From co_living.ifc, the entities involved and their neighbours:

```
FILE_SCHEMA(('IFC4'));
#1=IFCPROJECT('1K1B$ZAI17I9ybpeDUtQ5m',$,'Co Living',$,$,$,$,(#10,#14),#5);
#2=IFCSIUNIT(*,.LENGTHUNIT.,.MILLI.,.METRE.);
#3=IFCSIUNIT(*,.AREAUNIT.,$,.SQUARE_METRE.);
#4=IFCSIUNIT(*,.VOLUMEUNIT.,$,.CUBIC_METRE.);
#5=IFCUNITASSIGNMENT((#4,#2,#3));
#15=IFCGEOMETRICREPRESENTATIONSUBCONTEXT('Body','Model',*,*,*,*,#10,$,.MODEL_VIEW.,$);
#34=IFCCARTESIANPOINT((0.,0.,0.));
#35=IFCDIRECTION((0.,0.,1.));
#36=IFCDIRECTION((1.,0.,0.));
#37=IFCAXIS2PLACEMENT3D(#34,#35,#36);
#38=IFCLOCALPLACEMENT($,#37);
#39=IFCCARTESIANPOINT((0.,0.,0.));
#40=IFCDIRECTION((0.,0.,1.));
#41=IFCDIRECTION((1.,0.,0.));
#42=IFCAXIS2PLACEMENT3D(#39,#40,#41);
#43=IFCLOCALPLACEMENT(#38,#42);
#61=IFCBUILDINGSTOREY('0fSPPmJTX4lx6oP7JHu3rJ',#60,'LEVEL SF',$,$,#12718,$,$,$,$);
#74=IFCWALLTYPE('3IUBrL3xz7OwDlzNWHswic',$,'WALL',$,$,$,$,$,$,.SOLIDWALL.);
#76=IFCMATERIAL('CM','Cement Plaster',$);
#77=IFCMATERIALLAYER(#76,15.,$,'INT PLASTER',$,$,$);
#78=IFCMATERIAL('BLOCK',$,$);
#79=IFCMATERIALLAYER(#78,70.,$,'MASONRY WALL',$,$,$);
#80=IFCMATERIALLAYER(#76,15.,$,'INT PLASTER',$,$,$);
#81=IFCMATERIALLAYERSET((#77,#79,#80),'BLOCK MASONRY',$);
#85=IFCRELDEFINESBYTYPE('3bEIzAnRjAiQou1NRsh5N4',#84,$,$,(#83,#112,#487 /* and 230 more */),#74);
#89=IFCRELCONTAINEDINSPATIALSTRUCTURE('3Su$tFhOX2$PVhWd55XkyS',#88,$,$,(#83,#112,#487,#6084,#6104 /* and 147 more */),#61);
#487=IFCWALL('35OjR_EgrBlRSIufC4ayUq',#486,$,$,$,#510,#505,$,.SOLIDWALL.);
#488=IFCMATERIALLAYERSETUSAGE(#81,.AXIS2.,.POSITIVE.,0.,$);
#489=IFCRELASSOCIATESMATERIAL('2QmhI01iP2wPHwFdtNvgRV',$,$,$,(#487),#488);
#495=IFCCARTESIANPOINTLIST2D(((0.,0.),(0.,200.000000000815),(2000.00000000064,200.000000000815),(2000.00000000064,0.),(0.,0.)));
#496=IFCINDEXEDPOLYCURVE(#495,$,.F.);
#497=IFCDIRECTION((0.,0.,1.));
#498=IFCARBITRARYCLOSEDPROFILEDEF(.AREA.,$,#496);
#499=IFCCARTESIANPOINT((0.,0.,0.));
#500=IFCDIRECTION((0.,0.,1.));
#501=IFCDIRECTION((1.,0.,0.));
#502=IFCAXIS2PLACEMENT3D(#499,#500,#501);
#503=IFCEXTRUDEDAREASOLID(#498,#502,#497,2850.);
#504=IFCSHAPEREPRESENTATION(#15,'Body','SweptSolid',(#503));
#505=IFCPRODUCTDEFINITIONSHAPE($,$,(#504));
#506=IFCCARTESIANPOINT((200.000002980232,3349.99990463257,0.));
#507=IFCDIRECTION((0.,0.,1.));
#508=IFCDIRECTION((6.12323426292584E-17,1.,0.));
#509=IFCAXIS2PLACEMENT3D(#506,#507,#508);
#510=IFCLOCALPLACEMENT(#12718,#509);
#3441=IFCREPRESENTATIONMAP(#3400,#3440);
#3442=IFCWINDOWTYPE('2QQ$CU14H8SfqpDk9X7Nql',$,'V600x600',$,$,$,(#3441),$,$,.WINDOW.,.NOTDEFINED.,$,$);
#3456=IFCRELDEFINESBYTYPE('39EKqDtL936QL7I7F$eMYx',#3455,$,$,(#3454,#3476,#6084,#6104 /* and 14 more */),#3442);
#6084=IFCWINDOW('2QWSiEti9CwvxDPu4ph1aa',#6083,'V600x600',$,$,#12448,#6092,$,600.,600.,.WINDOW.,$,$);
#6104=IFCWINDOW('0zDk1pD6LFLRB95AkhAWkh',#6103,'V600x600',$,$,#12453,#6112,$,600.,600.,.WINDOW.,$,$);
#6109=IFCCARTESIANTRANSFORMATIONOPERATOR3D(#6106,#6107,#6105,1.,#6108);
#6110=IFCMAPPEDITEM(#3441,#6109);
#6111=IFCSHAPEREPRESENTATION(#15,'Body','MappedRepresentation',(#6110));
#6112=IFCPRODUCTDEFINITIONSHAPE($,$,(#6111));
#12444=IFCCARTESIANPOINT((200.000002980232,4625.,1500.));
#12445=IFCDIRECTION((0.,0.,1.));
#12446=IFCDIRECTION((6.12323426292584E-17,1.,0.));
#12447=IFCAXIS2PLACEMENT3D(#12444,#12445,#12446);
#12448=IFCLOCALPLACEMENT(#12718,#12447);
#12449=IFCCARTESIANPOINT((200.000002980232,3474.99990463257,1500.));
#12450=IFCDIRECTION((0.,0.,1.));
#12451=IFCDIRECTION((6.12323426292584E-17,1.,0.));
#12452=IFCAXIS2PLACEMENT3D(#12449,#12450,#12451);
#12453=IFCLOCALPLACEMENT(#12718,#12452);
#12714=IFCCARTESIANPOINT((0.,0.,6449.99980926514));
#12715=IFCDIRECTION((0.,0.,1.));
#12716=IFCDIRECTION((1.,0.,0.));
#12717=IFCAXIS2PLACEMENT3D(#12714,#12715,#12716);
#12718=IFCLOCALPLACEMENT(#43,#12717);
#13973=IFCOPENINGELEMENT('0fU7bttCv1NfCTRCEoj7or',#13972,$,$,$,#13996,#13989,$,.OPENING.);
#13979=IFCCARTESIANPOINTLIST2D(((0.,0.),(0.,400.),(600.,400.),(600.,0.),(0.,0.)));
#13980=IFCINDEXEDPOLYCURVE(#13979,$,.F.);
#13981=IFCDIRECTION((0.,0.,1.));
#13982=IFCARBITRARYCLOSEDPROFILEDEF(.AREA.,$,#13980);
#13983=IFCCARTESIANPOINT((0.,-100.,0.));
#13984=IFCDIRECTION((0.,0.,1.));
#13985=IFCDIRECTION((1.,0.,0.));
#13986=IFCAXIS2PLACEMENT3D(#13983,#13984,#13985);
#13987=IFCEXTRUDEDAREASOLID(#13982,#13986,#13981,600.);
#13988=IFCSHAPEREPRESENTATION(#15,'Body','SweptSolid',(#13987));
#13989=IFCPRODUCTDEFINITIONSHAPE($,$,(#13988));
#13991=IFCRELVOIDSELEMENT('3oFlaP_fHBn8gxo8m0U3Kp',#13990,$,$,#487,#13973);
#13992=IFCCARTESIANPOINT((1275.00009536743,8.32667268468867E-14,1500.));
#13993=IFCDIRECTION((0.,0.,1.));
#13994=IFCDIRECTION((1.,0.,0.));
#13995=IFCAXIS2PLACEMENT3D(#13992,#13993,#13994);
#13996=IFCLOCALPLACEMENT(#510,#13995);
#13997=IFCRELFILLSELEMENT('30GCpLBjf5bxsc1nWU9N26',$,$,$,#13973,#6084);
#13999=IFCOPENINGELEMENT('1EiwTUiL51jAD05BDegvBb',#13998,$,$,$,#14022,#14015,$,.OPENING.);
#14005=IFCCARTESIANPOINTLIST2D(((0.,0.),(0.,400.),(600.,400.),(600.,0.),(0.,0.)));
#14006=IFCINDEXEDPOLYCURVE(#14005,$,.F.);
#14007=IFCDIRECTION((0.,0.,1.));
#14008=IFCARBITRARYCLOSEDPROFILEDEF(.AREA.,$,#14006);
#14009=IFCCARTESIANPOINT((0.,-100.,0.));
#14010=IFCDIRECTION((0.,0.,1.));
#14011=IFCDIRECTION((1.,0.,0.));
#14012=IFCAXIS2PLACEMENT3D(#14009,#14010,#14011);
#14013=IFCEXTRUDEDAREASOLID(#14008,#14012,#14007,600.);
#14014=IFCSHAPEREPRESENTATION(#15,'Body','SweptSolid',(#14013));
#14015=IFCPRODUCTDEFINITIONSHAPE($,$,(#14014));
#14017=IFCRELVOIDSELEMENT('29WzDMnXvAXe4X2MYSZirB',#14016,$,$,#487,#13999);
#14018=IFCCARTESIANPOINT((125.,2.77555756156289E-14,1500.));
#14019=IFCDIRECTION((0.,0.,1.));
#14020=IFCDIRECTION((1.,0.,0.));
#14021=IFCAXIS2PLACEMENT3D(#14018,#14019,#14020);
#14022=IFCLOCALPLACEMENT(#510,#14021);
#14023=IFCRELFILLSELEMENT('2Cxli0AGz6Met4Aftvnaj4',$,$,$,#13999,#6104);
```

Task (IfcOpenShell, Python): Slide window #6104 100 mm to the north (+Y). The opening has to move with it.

```python
import ifcopenshell
import ifcopenshell.api.geometry
import ifcopenshell.util.placement
import ifcopenshell.util.unit

model = ifcopenshell.open("co_living.ifc")
unit_scale = ifcopenshell.util.unit.calculate_unit_scale(model)

window = model.by_guid("0zDk1pD6LFLRB95AkhAWkh")
opening = window.FillsVoids[0].RelatingOpeningElement
wall = opening.VoidsElements[0].RelatingBuildingElement

wall_matrix = ifcopenshell.util.placement.get_local_placement(wall.ObjectPlacement)
shift = wall_matrix[:3, 0] * 0.1 / unit_scale
before = ifcopenshell.util.placement.get_local_placement(window.ObjectPlacement)[:3, 3].copy()

# The window is not placed relative to its opening, so move both.
for product in (opening, window):
    matrix = ifcopenshell.util.placement.get_local_placement(product.ObjectPlacement)
    matrix[:3, 3] += shift
    ifcopenshell.api.geometry.edit_object_placement(model, product=product, matrix=matrix, is_si=False)

after = ifcopenshell.util.placement.get_local_placement(window.ObjectPlacement)[:3, 3]
print("window moved by", (after - before).round(3) + 0.0)

model.write("co_living_v2.ifc")
```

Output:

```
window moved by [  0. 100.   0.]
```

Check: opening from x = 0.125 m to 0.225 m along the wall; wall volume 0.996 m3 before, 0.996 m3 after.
